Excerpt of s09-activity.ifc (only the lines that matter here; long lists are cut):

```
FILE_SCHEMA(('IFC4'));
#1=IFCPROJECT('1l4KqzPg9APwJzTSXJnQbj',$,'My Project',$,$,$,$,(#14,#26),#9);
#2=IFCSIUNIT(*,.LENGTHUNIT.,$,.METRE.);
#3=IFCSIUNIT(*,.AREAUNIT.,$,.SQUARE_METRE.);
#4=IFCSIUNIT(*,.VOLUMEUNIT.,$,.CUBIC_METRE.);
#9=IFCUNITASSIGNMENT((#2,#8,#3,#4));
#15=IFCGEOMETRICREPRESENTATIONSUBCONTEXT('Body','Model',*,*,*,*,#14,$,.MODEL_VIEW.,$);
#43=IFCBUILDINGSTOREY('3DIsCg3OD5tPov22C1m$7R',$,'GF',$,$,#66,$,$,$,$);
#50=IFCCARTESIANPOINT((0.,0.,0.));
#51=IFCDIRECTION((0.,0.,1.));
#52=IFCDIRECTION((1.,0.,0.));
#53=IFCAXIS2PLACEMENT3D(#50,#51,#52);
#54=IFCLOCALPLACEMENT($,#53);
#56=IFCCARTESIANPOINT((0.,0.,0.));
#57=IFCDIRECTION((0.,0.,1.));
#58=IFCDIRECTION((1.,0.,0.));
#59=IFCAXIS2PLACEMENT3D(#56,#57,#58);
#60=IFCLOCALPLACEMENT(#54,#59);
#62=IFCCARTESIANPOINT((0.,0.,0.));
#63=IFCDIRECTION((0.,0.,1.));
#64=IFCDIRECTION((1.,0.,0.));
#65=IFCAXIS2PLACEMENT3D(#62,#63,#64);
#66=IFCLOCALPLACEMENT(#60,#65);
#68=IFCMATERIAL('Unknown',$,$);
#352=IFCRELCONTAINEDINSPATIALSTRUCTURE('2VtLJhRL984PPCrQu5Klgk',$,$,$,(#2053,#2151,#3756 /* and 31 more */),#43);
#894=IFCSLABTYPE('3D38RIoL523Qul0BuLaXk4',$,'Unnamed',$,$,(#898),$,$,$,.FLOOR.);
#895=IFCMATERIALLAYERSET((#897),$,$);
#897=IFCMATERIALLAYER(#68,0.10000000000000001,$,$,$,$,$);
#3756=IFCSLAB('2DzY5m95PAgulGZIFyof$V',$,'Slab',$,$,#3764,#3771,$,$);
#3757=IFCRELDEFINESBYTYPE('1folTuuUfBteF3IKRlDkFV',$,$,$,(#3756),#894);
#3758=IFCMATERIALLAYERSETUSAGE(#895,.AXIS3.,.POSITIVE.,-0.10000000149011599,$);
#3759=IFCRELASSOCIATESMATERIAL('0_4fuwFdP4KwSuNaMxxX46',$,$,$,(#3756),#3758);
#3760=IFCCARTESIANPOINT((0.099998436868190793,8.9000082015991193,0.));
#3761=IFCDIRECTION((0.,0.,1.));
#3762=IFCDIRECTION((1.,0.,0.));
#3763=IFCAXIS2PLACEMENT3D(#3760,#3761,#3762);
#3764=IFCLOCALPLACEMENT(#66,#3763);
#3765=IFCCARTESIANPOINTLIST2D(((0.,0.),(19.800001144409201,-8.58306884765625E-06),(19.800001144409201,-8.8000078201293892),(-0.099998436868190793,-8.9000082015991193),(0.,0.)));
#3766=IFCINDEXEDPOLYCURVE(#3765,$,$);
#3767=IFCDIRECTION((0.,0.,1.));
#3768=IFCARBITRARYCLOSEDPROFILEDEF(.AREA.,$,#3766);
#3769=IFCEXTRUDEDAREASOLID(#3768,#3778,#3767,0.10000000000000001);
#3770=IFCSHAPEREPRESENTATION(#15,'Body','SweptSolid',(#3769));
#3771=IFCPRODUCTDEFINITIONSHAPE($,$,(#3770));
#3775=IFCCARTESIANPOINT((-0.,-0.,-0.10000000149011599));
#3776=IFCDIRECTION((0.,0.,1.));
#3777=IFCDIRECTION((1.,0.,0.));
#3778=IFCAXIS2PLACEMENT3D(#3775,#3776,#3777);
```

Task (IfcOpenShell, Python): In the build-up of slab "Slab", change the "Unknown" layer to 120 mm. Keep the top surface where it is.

```python
import ifcopenshell
import ifcopenshell.util.element
import ifcopenshell.util.representation

model = ifcopenshell.open("s09-activity.ifc")

layer_set = model.by_id(895)
layer = next(l for l in layer_set.MaterialLayers if l.Material and l.Material.Name == "Unknown")
change = 0.12 - layer.LayerThickness
layer.LayerThickness += change

# Geometry does not follow the layer set by itself.
slabs = [e for e in ifcopenshell.util.element.get_elements_by_material(model, layer_set) if e.is_a("IfcSlab")]
for slab in sorted(slabs, key=lambda e: e.id()):
    body = ifcopenshell.util.representation.get_representation(slab, "Model", "Body")
    solid = body.Items[0]
    old_depth = solid.Depth
    solid.Depth += change
    # Extruded upwards: lower the start of the extrusion so the top stays.
    x, y, z = solid.Position.Location.Coordinates
    solid.Position.Location = model.createIfcCartesianPoint((x, y, z - change))
    print(slab.id(), f"{old_depth:g} -> {solid.Depth:g}")

# The layers are counted up from the underside, which has moved.
for usage in {ifcopenshell.util.element.get_material(slab) for slab in slabs}:
    usage.OffsetFromReferenceLine -= change

model.write("s09-activity_v2.ifc")
```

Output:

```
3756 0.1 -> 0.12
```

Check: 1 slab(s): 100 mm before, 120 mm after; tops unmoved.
